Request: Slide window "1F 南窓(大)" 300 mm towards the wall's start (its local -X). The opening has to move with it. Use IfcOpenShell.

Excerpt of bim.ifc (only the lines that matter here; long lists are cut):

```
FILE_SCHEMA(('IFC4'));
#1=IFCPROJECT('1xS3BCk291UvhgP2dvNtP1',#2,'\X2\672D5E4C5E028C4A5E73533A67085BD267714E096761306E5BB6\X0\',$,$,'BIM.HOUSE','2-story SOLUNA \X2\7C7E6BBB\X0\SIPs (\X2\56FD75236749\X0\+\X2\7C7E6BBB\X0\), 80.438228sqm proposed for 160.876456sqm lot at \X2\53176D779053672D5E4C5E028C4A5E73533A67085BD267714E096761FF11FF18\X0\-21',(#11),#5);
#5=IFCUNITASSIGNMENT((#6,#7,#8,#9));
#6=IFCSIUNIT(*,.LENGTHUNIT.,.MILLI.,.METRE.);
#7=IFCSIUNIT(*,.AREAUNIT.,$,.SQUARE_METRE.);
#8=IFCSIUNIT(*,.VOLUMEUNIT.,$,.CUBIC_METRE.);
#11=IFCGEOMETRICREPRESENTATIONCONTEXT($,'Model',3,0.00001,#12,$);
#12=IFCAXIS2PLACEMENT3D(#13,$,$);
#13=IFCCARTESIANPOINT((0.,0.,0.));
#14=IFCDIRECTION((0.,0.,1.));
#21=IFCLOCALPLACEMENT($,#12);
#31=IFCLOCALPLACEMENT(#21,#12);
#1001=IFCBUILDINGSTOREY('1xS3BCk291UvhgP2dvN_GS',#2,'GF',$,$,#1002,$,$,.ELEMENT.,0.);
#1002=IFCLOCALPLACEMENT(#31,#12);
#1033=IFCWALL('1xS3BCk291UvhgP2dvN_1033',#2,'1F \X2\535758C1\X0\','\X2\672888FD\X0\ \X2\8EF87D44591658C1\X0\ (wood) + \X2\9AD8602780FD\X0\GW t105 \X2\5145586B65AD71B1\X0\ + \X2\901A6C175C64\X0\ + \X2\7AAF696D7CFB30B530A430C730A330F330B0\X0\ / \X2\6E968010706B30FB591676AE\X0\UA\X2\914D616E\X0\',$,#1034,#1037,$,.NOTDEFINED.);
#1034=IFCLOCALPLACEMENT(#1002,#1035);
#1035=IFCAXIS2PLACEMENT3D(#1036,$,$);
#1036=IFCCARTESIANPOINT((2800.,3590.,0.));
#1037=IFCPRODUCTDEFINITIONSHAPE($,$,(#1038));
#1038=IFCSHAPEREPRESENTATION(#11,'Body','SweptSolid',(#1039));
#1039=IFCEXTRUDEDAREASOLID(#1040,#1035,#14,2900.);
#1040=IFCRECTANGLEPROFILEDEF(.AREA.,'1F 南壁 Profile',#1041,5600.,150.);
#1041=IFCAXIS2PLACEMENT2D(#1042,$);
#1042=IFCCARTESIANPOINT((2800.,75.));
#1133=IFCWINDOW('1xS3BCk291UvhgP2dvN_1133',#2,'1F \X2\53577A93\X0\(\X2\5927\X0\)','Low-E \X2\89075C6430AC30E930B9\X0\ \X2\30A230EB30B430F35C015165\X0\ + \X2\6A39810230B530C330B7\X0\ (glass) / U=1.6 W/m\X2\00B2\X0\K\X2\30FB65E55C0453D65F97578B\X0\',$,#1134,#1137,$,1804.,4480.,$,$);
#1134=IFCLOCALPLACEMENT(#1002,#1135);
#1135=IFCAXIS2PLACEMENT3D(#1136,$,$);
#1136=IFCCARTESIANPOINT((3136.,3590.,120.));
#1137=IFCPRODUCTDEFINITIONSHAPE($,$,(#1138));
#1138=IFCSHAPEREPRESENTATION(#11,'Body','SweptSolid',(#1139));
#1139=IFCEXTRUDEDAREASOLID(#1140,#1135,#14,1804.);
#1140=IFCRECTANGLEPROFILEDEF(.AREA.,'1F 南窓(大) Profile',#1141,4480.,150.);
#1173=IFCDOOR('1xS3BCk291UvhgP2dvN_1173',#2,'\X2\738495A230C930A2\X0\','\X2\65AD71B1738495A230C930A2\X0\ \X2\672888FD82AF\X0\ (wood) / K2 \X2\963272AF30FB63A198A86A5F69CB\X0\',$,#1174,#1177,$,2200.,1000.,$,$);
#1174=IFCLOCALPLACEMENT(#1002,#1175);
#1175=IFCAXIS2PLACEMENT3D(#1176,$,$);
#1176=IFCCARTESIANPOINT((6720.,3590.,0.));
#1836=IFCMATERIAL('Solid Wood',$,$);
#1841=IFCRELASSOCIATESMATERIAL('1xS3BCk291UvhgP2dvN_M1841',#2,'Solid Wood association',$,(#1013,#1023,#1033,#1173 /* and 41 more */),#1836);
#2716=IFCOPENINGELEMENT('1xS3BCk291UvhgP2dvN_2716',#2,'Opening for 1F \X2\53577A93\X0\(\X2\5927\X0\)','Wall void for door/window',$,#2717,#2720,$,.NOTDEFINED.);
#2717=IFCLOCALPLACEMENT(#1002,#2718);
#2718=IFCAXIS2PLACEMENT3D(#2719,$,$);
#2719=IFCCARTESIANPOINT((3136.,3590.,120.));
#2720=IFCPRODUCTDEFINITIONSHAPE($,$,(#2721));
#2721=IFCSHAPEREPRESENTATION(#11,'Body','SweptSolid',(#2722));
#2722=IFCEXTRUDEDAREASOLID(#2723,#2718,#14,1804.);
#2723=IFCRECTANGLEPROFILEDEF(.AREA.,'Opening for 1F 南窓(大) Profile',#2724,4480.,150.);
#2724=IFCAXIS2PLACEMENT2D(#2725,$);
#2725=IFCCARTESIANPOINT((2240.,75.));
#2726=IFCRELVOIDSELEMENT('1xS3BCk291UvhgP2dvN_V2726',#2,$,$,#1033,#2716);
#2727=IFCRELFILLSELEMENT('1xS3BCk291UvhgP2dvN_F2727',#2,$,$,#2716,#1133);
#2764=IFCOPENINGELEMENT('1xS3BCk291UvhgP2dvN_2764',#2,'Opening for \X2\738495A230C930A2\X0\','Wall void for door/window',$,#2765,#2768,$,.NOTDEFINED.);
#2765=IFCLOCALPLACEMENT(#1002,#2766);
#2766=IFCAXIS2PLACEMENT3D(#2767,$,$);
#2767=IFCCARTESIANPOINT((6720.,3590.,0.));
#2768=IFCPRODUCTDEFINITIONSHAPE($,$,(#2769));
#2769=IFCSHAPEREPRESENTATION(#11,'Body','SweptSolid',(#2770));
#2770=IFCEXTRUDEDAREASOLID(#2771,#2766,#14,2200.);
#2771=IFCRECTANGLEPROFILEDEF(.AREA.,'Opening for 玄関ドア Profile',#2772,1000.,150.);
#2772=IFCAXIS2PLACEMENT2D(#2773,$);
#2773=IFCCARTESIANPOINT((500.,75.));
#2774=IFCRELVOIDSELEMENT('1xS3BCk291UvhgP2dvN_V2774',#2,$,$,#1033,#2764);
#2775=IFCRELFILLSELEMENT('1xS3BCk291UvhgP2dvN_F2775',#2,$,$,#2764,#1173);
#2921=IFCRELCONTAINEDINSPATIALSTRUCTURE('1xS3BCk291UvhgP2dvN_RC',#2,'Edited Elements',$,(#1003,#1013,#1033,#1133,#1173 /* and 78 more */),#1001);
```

```python
import ifcopenshell
import ifcopenshell.api.geometry
import ifcopenshell.util.placement

model = ifcopenshell.open("bim.ifc")

window = model.by_guid("1xS3BCk291UvhgP2dvN_1133")
opening = window.FillsVoids[0].RelatingOpeningElement
wall = opening.VoidsElements[0].RelatingBuildingElement

wall_matrix = ifcopenshell.util.placement.get_local_placement(wall.ObjectPlacement)
shift = wall_matrix[:3, 0] * -300.0
before = ifcopenshell.util.placement.get_local_placement(window.ObjectPlacement)[:3, 3].copy()

# The window is not placed relative to its opening, so move both.
for product in (opening, window):
    matrix = ifcopenshell.util.placement.get_local_placement(product.ObjectPlacement)
    matrix[:3, 3] += shift
    ifcopenshell.api.geometry.edit_object_placement(model, product=product, matrix=matrix, is_si=False)

after = ifcopenshell.util.placement.get_local_placement(window.ObjectPlacement)[:3, 3]
print("window moved by", (after - before).round(3) + 0.0)

model.write("bim_v2.ifc")
```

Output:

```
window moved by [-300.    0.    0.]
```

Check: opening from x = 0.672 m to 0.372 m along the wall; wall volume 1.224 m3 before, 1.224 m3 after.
